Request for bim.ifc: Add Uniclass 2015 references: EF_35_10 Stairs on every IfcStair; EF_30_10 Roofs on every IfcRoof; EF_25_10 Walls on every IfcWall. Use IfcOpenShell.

First a look at what the model holds.

```python
import ifcopenshell

model = ifcopenshell.open("bim.ifc")
print(model.schema)
print("classifications:", [c.Name for c in model.by_type("IfcClassification")])
for ifc_class in ("IfcDoor", "IfcRoof", "IfcStair", "IfcWall", "IfcWindow"):
    print(ifc_class, len(model.by_type(ifc_class)))
```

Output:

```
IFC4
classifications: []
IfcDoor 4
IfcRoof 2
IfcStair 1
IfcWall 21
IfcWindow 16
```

```python
import ifcopenshell
import ifcopenshell.api.classification

model = ifcopenshell.open("bim.ifc")

system = ifcopenshell.api.classification.add_classification(model, classification="Uniclass 2015")

codes = {
    "IfcStair": ("EF_35_10", "Stairs"),
    "IfcRoof": ("EF_30_10", "Roofs"),
    "IfcWall": ("EF_25_10", "Walls"),
}
for ifc_class, (code, name) in codes.items():
    products = model.by_type(ifc_class)
    ifcopenshell.api.classification.add_reference(
        model, products=products, classification=system, identification=code, name=name
    )
    print(code, len(products))

model.write("bim_rev.ifc")
```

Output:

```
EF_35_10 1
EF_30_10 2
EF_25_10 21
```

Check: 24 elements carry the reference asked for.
